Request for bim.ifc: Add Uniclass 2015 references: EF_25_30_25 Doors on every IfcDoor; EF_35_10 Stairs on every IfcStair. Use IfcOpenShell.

First a look at what the model holds.

```python
import ifcopenshell

model = ifcopenshell.open("bim.ifc")
print(model.schema)
print("classifications:", [c.Name for c in model.by_type("IfcClassification")])
for ifc_class in ("IfcDoor", "IfcRoof", "IfcStair", "IfcWall", "IfcWindow"):
    print(ifc_class, len(model.by_type(ifc_class)))
```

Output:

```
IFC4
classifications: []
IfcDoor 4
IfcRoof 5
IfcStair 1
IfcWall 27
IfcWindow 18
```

```python
import ifcopenshell
import ifcopenshell.api.classification

model = ifcopenshell.open("bim.ifc")

system = ifcopenshell.api.classification.add_classification(model, classification="Uniclass 2015")

codes = {
    "IfcDoor": ("EF_25_30_25", "Doors"),
    "IfcStair": ("EF_35_10", "Stairs"),
}
for ifc_class, (code, name) in codes.items():
    products = model.by_type(ifc_class)
    ifcopenshell.api.classification.add_reference(
        model, products=products, classification=system, identification=code, name=name
    )
    print(code, len(products))

model.write("bim-out.ifc")
```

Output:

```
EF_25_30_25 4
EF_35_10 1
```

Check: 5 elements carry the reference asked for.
